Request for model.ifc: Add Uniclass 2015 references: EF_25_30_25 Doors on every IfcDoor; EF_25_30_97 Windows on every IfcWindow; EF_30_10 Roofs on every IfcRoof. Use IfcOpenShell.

First a look at what the model holds.

```python
import ifcopenshell

model = ifcopenshell.open("model.ifc")
print(model.schema)
print("classifications:", [c.Name for c in model.by_type("IfcClassification")])
for ifc_class in ("IfcDoor", "IfcRoof", "IfcStair", "IfcWall", "IfcWindow"):
    print(ifc_class, len(model.by_type(ifc_class)))
```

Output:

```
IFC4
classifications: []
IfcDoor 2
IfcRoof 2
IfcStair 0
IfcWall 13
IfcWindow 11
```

```python
import ifcopenshell
import ifcopenshell.api.classification

model = ifcopenshell.open("model.ifc")

system = ifcopenshell.api.classification.add_classification(model, classification="Uniclass 2015")

codes = {
    "IfcDoor": ("EF_25_30_25", "Doors"),
    "IfcWindow": ("EF_25_30_97", "Windows"),
    "IfcRoof": ("EF_30_10", "Roofs"),
}
for ifc_class, (code, name) in codes.items():
    products = model.by_type(ifc_class)
    ifcopenshell.api.classification.add_reference(
        model, products=products, classification=system, identification=code, name=name
    )
    print(code, len(products))

model.write("model_updated.ifc")
```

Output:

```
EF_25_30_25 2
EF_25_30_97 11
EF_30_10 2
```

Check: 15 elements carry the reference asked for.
